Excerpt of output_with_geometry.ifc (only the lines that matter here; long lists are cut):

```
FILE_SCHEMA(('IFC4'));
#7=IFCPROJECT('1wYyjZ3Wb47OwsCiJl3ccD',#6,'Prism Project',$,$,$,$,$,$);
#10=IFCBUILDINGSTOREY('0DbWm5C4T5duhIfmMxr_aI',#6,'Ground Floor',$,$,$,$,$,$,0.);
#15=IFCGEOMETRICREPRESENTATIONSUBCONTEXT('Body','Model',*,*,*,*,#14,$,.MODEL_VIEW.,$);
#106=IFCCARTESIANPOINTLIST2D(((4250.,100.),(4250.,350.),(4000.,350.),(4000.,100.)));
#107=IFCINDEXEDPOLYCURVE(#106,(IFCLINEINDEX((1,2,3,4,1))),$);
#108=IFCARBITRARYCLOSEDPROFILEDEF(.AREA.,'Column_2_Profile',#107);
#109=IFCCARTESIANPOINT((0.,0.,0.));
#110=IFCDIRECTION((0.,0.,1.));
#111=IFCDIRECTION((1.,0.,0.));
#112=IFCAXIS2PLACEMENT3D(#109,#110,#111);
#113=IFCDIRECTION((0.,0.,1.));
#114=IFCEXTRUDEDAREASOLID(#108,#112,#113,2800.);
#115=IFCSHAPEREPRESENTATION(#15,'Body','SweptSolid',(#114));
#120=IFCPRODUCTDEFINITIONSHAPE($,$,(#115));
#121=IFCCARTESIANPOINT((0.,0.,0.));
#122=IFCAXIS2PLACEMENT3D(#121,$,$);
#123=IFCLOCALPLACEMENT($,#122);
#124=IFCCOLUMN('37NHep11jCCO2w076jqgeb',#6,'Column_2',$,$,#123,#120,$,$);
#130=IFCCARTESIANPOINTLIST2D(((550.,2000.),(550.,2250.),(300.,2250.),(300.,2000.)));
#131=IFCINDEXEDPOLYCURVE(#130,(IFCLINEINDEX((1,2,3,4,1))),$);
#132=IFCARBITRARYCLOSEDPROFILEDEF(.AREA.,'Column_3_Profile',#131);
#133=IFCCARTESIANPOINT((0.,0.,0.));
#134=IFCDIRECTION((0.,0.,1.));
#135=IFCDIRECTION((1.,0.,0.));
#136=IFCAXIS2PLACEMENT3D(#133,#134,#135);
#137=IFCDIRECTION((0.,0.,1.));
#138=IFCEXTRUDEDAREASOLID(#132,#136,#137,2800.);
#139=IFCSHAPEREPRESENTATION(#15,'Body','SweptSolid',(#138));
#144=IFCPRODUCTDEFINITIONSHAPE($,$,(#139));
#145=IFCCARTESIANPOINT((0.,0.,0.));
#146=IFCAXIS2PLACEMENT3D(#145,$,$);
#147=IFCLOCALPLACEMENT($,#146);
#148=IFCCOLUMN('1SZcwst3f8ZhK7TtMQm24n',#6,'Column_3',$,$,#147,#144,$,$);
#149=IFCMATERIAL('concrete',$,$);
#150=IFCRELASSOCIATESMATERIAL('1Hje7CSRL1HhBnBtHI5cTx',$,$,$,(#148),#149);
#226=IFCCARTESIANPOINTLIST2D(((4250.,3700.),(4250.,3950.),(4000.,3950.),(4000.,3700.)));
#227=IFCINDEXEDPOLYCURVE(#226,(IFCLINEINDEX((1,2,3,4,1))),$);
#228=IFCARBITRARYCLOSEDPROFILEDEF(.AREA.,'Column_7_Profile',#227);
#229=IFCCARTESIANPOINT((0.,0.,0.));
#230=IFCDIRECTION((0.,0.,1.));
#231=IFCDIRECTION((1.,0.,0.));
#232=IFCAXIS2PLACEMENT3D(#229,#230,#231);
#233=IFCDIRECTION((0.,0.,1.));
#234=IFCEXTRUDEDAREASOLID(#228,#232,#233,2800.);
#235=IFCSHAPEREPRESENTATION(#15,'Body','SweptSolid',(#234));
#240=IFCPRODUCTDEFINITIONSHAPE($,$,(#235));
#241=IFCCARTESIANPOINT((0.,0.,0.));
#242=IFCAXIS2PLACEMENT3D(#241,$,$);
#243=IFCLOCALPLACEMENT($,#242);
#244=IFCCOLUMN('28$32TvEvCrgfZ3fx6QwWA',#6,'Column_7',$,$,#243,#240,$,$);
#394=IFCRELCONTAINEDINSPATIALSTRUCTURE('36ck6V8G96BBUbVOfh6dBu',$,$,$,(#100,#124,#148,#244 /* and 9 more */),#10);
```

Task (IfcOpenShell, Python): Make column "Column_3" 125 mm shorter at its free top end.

```python
import ifcopenshell
import ifcopenshell.util.representation
import ifcopenshell.util.unit

model = ifcopenshell.open("output_with_geometry.ifc")
unit_scale = ifcopenshell.util.unit.calculate_unit_scale(model)

member = model.by_guid("1SZcwst3f8ZhK7TtMQm24n")
change = -0.125 / unit_scale

# The extrusion runs towards the end named, so only its depth changes.
body = ifcopenshell.util.representation.get_representation(member, "Model", "Body")
solid = body.Items[0]
old_length = solid.Depth
solid.Depth += change

print(f"length {old_length:g} -> {solid.Depth:g}")

model.write("output_with_geometry_rev.ifc")
```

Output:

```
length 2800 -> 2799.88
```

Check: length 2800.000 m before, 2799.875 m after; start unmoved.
